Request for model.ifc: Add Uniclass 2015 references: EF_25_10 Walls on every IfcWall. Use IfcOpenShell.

First a look at what the model holds.

```python
import ifcopenshell

model = ifcopenshell.open("model.ifc")
print(model.schema)
print("classifications:", [c.Name for c in model.by_type("IfcClassification")])
for ifc_class in ("IfcDoor", "IfcRoof", "IfcStair", "IfcWall", "IfcWindow"):
    print(ifc_class, len(model.by_type(ifc_class)))
```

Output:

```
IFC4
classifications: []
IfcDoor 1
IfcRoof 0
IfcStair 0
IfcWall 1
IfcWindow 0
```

```python
import ifcopenshell
import ifcopenshell.api.classification

model = ifcopenshell.open("model.ifc")

system = ifcopenshell.api.classification.add_classification(model, classification="Uniclass 2015")

codes = {
    "IfcWall": ("EF_25_10", "Walls"),
}
for ifc_class, (code, name) in codes.items():
    products = model.by_type(ifc_class)
    ifcopenshell.api.classification.add_reference(
        model, products=products, classification=system, identification=code, name=name
    )
    print(code, len(products))

model.write("model_v2.ifc")
```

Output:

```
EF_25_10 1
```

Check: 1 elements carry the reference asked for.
